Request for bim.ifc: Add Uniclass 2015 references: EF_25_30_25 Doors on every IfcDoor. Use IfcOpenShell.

First a look at what the model holds.

```python
import ifcopenshell

model = ifcopenshell.open("bim.ifc")
print(model.schema)
print("classifications:", [c.Name for c in model.by_type("IfcClassification")])
for ifc_class in ("IfcDoor", "IfcRoof", "IfcStair", "IfcWall", "IfcWindow"):
    print(ifc_class, len(model.by_type(ifc_class)))
```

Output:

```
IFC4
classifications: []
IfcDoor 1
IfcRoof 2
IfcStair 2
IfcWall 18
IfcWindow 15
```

```python
import ifcopenshell
import ifcopenshell.api.classification

model = ifcopenshell.open("bim.ifc")

system = ifcopenshell.api.classification.add_classification(model, classification="Uniclass 2015")

codes = {
    "IfcDoor": ("EF_25_30_25", "Doors"),
}
for ifc_class, (code, name) in codes.items():
    products = model.by_type(ifc_class)
    ifcopenshell.api.classification.add_reference(
        model, products=products, classification=system, identification=code, name=name
    )
    print(code, len(products))

model.write("bim-out.ifc")
```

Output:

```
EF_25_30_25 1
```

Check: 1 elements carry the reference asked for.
